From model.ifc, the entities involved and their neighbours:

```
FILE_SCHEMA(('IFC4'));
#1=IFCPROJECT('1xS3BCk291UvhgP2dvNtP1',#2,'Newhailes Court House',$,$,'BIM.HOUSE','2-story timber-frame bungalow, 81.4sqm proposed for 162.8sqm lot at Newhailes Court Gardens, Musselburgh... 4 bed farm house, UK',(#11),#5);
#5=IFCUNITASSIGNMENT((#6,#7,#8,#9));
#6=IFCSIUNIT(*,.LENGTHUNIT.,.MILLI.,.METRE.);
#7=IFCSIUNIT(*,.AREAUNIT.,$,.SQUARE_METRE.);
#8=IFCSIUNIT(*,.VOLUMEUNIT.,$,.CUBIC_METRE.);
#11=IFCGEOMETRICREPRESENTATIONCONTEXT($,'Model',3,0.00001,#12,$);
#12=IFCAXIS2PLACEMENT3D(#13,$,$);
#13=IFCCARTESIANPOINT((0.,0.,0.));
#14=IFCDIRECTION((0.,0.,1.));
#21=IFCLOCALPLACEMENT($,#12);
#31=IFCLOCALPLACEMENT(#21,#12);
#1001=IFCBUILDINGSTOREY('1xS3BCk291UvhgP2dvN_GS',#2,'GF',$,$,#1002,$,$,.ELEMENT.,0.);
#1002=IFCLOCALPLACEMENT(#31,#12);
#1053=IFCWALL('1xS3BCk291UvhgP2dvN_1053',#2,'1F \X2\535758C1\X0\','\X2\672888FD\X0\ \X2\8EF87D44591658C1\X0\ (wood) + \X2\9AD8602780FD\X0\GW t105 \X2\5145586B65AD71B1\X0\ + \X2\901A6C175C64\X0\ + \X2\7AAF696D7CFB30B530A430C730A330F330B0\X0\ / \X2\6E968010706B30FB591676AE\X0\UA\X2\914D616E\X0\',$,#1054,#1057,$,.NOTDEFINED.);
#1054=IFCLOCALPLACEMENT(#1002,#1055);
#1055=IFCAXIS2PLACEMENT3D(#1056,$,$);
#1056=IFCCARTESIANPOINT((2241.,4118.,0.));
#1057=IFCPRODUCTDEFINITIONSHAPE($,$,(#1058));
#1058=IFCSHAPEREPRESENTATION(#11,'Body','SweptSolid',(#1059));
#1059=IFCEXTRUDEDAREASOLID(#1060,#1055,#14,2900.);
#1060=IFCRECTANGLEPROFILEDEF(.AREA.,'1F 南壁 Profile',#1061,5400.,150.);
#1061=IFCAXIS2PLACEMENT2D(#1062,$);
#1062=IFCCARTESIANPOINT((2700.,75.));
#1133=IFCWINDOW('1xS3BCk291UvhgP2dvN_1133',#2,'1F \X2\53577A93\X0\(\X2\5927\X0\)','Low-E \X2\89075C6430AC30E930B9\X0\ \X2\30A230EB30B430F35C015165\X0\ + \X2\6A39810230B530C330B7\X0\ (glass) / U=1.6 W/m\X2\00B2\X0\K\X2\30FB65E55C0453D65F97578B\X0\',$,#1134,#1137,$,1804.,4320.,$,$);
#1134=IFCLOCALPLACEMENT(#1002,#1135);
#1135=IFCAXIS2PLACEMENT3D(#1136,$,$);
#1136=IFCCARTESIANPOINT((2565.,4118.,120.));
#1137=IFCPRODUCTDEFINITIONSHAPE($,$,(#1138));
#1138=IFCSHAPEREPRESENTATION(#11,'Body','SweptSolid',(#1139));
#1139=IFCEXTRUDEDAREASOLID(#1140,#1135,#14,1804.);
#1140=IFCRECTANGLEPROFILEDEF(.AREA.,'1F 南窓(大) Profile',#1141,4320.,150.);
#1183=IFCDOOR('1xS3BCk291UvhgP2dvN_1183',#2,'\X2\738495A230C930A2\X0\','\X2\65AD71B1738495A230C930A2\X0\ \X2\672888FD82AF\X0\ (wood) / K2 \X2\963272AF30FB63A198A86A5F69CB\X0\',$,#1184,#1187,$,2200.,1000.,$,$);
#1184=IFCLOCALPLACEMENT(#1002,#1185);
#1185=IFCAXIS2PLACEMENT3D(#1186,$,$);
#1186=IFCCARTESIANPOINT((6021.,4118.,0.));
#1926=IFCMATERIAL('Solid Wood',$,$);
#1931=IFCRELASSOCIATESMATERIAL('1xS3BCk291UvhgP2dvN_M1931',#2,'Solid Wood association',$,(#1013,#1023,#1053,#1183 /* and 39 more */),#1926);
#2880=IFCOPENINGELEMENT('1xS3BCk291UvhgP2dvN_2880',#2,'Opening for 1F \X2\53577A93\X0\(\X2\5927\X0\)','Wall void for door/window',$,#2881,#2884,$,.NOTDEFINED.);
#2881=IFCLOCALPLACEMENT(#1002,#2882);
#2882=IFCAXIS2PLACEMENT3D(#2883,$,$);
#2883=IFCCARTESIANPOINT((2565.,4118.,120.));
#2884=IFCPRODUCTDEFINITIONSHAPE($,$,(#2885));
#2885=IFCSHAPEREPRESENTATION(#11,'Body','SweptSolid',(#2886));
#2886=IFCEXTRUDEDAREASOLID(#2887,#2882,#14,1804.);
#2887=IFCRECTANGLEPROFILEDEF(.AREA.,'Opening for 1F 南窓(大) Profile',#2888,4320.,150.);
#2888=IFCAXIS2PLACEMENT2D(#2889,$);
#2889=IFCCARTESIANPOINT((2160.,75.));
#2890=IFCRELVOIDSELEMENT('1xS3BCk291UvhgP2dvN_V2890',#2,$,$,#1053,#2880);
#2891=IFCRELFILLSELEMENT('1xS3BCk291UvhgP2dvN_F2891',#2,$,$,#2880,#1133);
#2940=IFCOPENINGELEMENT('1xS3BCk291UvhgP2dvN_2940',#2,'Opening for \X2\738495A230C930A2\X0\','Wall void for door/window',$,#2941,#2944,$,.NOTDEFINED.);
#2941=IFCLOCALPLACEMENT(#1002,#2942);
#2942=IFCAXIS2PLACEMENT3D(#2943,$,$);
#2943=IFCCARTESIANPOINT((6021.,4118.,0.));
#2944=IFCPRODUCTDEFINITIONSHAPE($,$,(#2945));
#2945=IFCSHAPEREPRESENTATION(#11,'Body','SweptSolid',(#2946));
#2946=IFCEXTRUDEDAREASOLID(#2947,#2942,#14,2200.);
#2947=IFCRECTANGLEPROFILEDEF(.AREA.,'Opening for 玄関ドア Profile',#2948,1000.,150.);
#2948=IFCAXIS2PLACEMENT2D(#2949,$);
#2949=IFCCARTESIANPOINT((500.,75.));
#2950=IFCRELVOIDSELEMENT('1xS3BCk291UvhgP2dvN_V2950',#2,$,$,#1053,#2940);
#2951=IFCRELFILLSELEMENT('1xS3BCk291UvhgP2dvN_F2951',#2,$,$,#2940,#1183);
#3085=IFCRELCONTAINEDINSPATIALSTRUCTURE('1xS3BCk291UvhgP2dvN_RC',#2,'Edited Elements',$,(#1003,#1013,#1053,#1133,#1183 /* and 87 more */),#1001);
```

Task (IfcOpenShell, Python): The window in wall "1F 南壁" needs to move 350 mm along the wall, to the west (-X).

```python
import ifcopenshell
import ifcopenshell.api.geometry
import ifcopenshell.util.placement
import ifcopenshell.util.unit

model = ifcopenshell.open("model.ifc")
unit_scale = ifcopenshell.util.unit.calculate_unit_scale(model)

window = model.by_id(1133)
opening = window.FillsVoids[0].RelatingOpeningElement
wall = opening.VoidsElements[0].RelatingBuildingElement

wall_matrix = ifcopenshell.util.placement.get_local_placement(wall.ObjectPlacement)
shift = wall_matrix[:3, 0] * -0.35 / unit_scale
before = ifcopenshell.util.placement.get_local_placement(window.ObjectPlacement)[:3, 3].copy()

# The window is not placed relative to its opening, so move both.
for product in (opening, window):
    matrix = ifcopenshell.util.placement.get_local_placement(product.ObjectPlacement)
    matrix[:3, 3] += shift
    ifcopenshell.api.geometry.edit_object_placement(model, product=product, matrix=matrix, is_si=False)

after = ifcopenshell.util.placement.get_local_placement(window.ObjectPlacement)[:3, 3]
print("window moved by", (after - before).round(3) + 0.0)

model.write("model_v2.ifc")
```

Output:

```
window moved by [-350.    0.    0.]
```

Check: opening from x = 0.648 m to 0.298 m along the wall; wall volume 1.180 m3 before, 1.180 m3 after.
